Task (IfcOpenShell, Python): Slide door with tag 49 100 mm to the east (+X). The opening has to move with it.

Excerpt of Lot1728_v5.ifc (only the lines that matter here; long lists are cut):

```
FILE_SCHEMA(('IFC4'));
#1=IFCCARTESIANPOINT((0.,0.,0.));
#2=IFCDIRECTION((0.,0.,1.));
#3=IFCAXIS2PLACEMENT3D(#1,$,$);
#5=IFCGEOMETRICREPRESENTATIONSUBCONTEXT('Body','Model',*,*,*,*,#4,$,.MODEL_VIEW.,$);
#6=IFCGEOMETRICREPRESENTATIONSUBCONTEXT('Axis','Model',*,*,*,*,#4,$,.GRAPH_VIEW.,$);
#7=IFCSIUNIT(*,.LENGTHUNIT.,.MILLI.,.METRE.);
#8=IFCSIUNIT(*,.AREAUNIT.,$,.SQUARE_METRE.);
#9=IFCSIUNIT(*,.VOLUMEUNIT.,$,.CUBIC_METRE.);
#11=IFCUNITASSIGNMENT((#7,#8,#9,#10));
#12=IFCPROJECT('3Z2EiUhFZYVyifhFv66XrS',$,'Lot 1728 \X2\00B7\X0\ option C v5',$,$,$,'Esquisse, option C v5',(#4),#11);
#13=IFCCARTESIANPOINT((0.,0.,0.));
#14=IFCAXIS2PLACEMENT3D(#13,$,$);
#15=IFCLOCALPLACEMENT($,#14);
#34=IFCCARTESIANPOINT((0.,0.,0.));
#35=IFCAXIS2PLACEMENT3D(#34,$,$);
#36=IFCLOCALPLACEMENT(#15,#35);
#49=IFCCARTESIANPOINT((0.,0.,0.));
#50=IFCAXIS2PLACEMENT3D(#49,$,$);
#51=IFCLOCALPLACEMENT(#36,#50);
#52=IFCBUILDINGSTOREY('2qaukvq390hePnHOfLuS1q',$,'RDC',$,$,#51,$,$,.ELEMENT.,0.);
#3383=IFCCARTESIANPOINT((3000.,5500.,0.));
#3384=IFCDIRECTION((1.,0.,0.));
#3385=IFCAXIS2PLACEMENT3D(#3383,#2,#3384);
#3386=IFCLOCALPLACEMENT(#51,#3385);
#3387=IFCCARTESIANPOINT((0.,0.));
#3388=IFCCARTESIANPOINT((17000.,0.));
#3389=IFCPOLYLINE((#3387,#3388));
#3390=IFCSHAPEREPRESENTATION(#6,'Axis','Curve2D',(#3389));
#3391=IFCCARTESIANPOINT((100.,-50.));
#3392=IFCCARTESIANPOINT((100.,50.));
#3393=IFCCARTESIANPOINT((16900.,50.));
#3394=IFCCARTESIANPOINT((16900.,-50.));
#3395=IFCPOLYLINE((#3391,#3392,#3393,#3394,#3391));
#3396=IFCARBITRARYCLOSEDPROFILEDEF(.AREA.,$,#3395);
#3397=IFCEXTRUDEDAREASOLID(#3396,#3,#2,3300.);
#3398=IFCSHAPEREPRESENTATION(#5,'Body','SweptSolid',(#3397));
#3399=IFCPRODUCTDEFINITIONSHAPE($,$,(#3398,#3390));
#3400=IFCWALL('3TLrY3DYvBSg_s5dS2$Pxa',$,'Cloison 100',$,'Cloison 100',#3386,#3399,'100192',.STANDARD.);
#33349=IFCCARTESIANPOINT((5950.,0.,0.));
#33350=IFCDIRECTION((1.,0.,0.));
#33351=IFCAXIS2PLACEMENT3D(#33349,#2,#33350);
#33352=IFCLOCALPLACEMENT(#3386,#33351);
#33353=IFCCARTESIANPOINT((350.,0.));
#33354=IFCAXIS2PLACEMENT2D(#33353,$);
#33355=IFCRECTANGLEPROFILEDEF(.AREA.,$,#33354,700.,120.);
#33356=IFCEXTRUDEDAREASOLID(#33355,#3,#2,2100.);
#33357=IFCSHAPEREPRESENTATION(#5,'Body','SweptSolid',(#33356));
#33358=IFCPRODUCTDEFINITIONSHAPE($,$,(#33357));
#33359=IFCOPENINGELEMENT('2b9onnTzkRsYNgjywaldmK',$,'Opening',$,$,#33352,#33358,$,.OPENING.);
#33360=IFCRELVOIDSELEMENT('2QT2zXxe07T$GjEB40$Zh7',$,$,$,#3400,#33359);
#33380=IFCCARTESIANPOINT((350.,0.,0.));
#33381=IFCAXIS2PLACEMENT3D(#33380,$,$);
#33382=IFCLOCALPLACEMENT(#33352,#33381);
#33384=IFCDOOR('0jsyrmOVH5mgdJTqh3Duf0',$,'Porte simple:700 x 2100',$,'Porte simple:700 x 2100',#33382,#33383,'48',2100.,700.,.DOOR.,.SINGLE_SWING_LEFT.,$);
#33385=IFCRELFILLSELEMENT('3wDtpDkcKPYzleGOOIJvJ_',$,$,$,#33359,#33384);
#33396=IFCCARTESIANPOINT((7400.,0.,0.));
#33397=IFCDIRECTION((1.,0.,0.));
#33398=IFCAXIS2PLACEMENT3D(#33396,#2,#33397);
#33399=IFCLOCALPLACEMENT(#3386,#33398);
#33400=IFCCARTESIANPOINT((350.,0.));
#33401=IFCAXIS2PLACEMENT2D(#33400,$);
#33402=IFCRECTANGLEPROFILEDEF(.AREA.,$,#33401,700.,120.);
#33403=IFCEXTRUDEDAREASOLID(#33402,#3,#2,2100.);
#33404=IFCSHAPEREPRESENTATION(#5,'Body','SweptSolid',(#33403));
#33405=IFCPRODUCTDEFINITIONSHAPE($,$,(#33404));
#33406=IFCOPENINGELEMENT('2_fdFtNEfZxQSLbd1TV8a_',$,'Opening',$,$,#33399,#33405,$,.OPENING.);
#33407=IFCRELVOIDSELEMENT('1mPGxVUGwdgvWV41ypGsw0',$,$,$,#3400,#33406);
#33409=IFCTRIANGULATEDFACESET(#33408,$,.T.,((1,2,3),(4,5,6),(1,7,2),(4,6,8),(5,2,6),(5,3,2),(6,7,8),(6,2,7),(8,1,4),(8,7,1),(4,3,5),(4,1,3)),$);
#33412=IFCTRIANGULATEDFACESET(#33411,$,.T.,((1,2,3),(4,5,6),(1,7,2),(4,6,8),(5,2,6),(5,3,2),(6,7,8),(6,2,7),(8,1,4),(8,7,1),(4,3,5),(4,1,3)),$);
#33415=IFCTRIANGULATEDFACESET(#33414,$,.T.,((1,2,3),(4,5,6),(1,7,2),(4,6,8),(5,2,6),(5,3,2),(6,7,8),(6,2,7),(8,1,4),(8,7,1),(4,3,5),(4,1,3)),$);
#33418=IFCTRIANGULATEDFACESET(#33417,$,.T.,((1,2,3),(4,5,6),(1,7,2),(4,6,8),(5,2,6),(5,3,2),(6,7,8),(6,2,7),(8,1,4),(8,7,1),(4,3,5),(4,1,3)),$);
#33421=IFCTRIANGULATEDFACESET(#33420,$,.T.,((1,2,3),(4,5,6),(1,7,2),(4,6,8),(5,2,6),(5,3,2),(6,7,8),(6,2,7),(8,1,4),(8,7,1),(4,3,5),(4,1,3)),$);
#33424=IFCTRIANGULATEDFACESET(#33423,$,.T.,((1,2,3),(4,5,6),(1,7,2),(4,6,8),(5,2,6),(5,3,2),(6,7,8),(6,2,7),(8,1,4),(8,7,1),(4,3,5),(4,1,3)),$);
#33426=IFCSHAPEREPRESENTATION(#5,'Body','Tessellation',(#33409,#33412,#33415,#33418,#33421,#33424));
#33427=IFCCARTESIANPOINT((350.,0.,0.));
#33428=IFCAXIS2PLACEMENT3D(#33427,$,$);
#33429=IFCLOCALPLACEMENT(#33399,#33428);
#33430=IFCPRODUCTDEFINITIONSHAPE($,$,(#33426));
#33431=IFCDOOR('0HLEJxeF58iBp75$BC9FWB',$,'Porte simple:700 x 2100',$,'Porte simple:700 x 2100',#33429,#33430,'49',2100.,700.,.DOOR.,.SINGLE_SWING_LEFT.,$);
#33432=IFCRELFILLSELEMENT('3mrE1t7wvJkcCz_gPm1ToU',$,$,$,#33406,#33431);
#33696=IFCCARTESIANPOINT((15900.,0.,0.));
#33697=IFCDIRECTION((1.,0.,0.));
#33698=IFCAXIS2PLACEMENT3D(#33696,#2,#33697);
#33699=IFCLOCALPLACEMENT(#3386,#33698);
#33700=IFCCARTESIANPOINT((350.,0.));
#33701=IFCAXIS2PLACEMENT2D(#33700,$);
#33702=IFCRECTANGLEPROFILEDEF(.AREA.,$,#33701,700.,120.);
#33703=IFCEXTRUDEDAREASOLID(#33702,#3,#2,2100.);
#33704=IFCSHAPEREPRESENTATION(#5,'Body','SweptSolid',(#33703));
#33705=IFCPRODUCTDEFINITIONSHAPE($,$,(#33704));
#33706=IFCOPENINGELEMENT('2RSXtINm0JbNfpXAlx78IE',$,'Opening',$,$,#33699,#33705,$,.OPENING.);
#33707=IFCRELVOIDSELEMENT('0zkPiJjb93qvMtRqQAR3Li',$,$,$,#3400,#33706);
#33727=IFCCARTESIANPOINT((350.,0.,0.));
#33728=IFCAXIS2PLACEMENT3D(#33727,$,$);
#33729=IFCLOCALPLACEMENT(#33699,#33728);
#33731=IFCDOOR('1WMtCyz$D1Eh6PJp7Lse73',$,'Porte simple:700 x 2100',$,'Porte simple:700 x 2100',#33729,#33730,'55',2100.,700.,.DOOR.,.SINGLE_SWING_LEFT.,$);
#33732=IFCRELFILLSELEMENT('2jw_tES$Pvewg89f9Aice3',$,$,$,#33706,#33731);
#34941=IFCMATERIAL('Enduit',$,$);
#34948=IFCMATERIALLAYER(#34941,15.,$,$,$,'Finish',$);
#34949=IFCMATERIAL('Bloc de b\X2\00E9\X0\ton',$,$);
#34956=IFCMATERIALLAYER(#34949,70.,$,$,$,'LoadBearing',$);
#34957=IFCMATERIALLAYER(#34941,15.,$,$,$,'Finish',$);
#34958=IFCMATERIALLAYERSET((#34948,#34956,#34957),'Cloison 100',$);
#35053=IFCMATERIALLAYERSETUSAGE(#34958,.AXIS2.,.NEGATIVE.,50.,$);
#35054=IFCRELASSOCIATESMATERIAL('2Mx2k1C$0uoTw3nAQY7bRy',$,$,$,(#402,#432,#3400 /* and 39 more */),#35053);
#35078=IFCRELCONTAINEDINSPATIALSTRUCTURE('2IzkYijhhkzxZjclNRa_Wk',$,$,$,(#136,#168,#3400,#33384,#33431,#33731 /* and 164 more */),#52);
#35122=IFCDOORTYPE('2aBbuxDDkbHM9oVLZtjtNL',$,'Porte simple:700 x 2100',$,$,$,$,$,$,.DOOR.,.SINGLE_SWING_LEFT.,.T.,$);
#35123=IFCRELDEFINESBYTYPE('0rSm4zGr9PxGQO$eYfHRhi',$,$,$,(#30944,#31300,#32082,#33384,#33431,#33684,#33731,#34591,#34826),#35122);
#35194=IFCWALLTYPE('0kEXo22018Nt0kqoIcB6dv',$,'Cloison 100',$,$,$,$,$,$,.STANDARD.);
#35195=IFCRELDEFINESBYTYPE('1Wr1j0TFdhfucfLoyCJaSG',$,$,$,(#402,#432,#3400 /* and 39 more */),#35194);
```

```python
import ifcopenshell
import ifcopenshell.api.geometry
import ifcopenshell.util.placement

model = ifcopenshell.open("Lot1728_v5.ifc")

door = model.by_guid("0HLEJxeF58iBp75$BC9FWB")
opening = door.FillsVoids[0].RelatingOpeningElement
wall = opening.VoidsElements[0].RelatingBuildingElement

wall_matrix = ifcopenshell.util.placement.get_local_placement(wall.ObjectPlacement)
shift = wall_matrix[:3, 0] * 100.0
before = ifcopenshell.util.placement.get_local_placement(door.ObjectPlacement)[:3, 3].copy()

# The door is placed relative to its opening, so it follows when the opening moves.
matrix = ifcopenshell.util.placement.get_local_placement(opening.ObjectPlacement)
matrix[:3, 3] += shift
ifcopenshell.api.geometry.edit_object_placement(
    model, product=opening, matrix=matrix, is_si=False, should_transform_children=True
)

after = ifcopenshell.util.placement.get_local_placement(door.ObjectPlacement)[:3, 3]
print("door moved by", (after - before).round(3) + 0.0)

model.write("Lot1728_v5_v2.ifc")
```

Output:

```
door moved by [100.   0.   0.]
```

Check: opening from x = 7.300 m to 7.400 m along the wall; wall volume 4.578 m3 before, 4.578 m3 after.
